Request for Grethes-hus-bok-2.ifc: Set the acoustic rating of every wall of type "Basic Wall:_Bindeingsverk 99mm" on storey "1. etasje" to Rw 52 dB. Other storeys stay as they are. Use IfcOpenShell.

First a look at what the model holds.

```python
import ifcopenshell
import ifcopenshell.util.element

model = ifcopenshell.open("Grethes-hus-bok-2.ifc")
print(model.schema)
storey = next(s for s in model.by_type("IfcBuildingStorey") if s.Name == "1. etasje")
walls = [e for e in ifcopenshell.util.element.get_decomposition(storey) if e.is_a("IfcWall")]
seen = {}
for e in walls:
    element_type = ifcopenshell.util.element.get_type(e)
    key = (element_type.Name if element_type != e and element_type else None, ifcopenshell.util.element.get_pset(e, "Pset_WallCommon", "AcousticRating"))
    seen[key] = seen.get(key, 0) + 1
for (name, value), count in sorted(seen.items(), key=str):
    print(count, "x", name, "|", value)
```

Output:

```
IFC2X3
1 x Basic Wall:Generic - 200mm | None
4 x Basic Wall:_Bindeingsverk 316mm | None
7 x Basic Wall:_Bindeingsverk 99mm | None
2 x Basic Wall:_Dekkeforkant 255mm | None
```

```python
import ifcopenshell
import ifcopenshell.api.pset
import ifcopenshell.util.element

model = ifcopenshell.open("Grethes-hus-bok-2.ifc")

storey = next(s for s in model.by_type("IfcBuildingStorey") if s.Name == "1. etasje")
walls = [e for e in ifcopenshell.util.element.get_decomposition(storey) if e.is_a("IfcWall")]

count = 0
for e in walls:
    element_type = ifcopenshell.util.element.get_type(e)
    if element_type in (None, e) or element_type.Name != "Basic Wall:_Bindeingsverk 99mm":
        continue
    # add_pset returns the element's existing set when there is one.
    pset = ifcopenshell.api.pset.add_pset(model, product=e, name="Pset_WallCommon")
    ifcopenshell.api.pset.edit_pset(model, pset=pset, properties={"AcousticRating": "Rw 52 dB"})
    count += 1

print(count, "walls updated")

model.write("Grethes-hus-bok-2_rev.ifc")
```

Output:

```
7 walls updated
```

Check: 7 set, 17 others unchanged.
